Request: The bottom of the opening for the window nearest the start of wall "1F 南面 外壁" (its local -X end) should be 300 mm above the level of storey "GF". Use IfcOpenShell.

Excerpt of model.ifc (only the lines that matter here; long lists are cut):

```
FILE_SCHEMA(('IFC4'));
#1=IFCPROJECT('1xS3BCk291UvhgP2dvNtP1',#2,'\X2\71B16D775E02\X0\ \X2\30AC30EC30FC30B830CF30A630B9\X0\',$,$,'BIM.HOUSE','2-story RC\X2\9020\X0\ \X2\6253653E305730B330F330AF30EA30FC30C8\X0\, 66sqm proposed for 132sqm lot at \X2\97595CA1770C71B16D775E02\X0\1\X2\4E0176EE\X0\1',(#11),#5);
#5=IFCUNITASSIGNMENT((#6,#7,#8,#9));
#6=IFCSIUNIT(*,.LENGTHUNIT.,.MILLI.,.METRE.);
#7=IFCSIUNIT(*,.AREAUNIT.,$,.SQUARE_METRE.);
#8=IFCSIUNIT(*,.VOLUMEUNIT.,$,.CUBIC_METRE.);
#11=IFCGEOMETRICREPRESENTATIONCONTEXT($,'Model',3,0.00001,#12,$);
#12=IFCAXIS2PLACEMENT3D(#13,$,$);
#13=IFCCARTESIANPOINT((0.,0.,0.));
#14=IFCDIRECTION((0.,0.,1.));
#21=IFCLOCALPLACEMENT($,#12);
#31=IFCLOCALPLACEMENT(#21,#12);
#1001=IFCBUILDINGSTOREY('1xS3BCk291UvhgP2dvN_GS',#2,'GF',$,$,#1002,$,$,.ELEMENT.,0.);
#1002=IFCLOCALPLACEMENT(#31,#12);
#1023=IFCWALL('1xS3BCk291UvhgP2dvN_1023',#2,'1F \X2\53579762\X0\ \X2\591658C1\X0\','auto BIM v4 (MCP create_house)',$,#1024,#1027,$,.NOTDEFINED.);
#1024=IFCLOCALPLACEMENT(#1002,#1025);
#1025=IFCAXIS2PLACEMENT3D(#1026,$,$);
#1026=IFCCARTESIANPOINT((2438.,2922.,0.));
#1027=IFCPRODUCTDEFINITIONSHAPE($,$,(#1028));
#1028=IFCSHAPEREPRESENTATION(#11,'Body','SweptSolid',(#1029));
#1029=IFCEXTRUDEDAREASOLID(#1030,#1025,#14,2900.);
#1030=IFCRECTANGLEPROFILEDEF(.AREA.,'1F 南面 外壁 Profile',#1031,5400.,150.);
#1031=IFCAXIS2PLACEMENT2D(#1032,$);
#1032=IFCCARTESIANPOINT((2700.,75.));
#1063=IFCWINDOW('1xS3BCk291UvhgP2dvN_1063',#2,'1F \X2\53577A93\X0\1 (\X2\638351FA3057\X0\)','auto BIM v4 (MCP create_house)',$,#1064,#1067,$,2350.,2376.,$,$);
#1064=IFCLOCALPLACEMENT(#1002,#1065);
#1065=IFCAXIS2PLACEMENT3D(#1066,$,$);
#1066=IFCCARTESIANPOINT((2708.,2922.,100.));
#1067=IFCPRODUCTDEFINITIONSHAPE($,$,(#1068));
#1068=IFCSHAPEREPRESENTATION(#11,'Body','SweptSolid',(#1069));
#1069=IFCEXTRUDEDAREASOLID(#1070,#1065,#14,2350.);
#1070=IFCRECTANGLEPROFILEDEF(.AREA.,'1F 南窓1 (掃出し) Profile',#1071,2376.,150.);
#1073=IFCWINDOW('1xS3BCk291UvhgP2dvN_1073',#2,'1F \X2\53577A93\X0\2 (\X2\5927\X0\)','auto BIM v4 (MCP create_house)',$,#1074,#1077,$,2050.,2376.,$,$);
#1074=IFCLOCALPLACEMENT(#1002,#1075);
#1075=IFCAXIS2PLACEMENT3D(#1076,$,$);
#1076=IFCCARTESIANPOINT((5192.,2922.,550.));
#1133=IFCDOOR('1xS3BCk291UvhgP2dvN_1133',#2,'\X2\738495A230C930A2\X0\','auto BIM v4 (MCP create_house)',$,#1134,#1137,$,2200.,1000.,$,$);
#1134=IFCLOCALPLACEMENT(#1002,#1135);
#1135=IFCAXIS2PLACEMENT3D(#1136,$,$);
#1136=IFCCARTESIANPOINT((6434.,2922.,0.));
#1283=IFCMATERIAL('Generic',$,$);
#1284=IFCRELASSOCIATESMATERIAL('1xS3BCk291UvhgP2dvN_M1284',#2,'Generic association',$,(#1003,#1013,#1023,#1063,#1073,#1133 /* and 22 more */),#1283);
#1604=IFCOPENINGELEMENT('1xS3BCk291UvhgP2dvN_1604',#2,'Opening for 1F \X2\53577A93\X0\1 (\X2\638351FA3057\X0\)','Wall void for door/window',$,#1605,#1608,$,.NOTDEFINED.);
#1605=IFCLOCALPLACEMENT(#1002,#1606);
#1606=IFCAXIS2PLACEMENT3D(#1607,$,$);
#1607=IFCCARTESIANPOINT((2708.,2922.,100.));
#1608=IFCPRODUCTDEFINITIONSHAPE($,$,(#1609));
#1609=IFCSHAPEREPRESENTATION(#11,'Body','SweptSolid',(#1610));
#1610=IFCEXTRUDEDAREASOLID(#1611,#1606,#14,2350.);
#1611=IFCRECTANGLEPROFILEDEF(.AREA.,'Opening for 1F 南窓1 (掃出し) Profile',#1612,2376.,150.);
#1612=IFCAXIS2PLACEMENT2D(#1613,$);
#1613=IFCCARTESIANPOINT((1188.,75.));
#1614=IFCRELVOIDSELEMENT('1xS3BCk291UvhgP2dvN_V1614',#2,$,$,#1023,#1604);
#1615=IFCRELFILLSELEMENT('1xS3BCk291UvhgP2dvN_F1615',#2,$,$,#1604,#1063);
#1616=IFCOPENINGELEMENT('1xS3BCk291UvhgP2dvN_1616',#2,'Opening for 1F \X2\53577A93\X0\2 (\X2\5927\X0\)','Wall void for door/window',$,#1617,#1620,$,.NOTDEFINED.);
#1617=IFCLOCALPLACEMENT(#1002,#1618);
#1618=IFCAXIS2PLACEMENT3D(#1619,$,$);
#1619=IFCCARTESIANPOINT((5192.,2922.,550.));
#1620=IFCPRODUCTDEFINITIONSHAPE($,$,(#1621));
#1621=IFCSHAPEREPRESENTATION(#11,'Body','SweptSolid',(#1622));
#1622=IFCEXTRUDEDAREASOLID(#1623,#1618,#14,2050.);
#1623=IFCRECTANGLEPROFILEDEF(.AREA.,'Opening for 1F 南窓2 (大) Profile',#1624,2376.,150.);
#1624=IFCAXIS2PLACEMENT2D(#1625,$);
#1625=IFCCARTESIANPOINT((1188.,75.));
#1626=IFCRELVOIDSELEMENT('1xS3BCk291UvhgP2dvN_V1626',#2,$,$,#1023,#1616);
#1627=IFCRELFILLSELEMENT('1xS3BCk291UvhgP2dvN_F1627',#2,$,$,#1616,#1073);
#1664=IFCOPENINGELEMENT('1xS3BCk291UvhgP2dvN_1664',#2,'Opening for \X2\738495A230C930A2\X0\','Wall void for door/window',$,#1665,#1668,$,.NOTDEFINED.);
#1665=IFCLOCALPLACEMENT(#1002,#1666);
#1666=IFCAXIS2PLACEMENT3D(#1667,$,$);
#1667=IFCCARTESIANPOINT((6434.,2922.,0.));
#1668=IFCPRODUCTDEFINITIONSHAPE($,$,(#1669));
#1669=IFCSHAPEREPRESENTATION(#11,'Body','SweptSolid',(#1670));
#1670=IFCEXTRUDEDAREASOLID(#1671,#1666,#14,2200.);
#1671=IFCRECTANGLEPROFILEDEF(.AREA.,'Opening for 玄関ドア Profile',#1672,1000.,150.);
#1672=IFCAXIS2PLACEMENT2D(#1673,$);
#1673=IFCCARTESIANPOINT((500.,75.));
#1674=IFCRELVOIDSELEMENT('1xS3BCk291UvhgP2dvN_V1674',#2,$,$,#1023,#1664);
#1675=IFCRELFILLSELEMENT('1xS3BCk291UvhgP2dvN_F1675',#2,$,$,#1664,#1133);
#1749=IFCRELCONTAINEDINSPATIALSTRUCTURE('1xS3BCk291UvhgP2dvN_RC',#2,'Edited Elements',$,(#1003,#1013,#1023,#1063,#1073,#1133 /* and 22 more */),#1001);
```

```python
import numpy as np
import ifcopenshell
import ifcopenshell.api.geometry
import ifcopenshell.geom
import ifcopenshell.util.element
import ifcopenshell.util.placement
import ifcopenshell.util.shape
import ifcopenshell.util.unit

model = ifcopenshell.open("model.ifc")
unit_scale = ifcopenshell.util.unit.calculate_unit_scale(model)

window = model.by_guid("1xS3BCk291UvhgP2dvN_1063")
opening = window.FillsVoids[0].RelatingOpeningElement
storey = ifcopenshell.util.element.get_container(window, ifc_class="IfcBuildingStorey")
level = ifcopenshell.util.placement.get_local_placement(storey.ObjectPlacement)[2, 3]

# The opening's origin need not be at the sill, so measure its lowest point.
shape = ifcopenshell.geom.create_shape(ifcopenshell.geom.settings(), opening)
bottom = ifcopenshell.util.shape.get_shape_bottom_elevation(shape, shape.geometry) / unit_scale
dz = level + 300.0 - bottom

shift = np.array([0.0, 0.0, dz])
# The window is not placed relative to its opening, so move both.
for product in (opening, window):
    matrix = ifcopenshell.util.placement.get_local_placement(product.ObjectPlacement)
    matrix[:3, 3] += shift
    ifcopenshell.api.geometry.edit_object_placement(model, product=product, matrix=matrix, is_si=False)

print(f"moved by {dz * unit_scale:+.3f} m")

model.write("model_v2.ifc")
```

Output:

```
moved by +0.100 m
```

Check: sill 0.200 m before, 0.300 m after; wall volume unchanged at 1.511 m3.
